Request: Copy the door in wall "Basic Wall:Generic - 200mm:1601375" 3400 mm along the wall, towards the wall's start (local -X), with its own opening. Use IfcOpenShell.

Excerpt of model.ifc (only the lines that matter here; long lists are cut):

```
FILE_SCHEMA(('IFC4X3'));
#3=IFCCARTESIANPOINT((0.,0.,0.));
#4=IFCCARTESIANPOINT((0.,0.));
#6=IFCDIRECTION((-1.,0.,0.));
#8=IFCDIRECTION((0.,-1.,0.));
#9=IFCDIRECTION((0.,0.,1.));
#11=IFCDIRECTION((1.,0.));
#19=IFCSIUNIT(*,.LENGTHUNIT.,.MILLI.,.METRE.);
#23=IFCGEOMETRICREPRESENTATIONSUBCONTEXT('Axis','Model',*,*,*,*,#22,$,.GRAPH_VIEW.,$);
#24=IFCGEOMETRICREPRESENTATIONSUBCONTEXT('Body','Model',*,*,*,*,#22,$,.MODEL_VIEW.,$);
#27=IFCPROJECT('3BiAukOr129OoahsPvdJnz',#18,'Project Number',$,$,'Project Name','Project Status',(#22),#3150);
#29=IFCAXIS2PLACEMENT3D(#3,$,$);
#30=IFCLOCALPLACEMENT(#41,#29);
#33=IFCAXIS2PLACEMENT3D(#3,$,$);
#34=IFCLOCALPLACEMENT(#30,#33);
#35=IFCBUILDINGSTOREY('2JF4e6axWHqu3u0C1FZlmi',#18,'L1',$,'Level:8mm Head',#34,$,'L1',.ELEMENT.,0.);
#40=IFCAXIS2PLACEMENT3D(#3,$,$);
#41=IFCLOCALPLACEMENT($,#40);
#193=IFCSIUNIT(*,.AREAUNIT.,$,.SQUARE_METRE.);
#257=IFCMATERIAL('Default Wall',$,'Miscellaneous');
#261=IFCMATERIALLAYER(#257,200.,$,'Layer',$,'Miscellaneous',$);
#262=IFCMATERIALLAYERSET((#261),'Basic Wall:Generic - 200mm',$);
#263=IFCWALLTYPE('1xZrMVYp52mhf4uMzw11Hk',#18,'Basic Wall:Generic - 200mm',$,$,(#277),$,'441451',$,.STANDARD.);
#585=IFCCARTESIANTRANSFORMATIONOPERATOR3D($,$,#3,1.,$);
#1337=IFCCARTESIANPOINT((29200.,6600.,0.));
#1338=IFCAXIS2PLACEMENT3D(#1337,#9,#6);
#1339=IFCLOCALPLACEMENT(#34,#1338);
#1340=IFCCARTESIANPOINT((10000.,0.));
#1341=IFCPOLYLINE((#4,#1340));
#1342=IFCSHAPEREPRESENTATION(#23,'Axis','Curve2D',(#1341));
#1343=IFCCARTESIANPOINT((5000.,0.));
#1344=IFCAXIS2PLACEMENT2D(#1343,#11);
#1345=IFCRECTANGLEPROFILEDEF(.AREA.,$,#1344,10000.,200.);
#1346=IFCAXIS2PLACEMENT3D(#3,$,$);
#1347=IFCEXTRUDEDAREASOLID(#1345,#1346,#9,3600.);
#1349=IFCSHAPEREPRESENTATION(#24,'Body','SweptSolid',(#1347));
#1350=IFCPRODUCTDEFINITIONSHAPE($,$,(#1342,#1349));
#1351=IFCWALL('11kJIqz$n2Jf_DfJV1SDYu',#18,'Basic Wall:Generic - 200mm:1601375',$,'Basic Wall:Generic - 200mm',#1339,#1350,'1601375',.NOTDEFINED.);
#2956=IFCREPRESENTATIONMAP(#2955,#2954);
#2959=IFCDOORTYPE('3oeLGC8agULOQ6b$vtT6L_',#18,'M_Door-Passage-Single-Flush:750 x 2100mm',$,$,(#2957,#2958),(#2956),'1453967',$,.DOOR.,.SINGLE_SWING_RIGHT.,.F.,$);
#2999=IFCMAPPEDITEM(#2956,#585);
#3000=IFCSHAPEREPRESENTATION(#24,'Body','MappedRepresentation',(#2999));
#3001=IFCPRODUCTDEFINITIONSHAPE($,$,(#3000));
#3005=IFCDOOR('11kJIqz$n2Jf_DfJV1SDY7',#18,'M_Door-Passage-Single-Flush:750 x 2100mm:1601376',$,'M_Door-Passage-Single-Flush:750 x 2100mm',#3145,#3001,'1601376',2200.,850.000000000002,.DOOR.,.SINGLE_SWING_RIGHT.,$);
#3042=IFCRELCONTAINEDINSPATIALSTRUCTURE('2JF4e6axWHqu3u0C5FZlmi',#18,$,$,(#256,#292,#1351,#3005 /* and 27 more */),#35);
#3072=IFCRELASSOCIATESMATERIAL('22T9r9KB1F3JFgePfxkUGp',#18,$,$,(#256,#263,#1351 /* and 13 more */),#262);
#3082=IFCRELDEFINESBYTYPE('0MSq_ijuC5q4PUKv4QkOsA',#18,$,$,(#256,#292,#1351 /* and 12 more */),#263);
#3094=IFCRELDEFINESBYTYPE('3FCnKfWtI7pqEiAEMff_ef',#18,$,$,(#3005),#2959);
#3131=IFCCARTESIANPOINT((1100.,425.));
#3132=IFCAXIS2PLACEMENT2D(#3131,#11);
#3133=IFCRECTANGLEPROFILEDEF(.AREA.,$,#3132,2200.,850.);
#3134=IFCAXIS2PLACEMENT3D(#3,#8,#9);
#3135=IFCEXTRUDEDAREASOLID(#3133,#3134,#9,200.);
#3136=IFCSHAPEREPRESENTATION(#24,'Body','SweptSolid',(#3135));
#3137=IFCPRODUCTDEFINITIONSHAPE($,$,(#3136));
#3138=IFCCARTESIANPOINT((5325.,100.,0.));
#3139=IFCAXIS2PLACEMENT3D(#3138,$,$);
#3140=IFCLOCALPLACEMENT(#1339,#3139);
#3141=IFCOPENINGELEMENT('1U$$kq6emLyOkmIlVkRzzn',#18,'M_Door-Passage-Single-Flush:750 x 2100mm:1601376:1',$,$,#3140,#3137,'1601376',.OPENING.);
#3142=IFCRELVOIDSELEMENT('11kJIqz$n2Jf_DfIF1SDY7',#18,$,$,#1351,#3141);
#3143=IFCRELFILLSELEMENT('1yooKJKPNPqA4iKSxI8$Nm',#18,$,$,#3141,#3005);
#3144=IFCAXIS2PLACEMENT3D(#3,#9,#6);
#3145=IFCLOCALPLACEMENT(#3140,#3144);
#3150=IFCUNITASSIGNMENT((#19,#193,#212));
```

```python
import ifcopenshell
import ifcopenshell.api.feature
import ifcopenshell.api.geometry
import ifcopenshell.api.root
import ifcopenshell.geom
import ifcopenshell.util.element
import ifcopenshell.util.placement
import ifcopenshell.util.shape

model = ifcopenshell.open("model.ifc")
settings = ifcopenshell.geom.settings()


def volume(element):
    """Net volume in cubic metres, openings subtracted."""
    shape = ifcopenshell.geom.create_shape(settings, element)
    return ifcopenshell.util.shape.get_volume(shape.geometry)


def reuse_history(source, copy):
    """copy_class also copies each property set's owner history, people and application; keep the originals."""
    for rel in copy.IsDefinedBy:
        if rel.is_a("IfcRelDefinesByProperties") and (history := rel.RelatingPropertyDefinition.OwnerHistory):
            rel.RelatingPropertyDefinition.OwnerHistory = source.OwnerHistory
            ifcopenshell.util.element.remove_deep2(model, history)


door = model.by_guid("11kJIqz$n2Jf_DfJV1SDY7")
opening = door.FillsVoids[0].RelatingOpeningElement
wall = opening.VoidsElements[0].RelatingBuildingElement
before = volume(wall)
shift = ifcopenshell.util.placement.get_local_placement(wall.ObjectPlacement)[:3, 0] * -3400.0

# copy_class copies the void relationship, type, container and properties, but no geometry.
new_opening = ifcopenshell.api.root.copy_class(model, product=opening)
new_opening.Representation = ifcopenshell.util.element.copy_deep(
    model, opening.Representation, exclude=["IfcGeometricRepresentationContext", "IfcRepresentationMap"]
)
new_opening.Name = "M_Door-Passage-Single-Flush:750 x 2100mm"
new_opening.Tag = None
new_door = ifcopenshell.api.root.copy_class(model, product=door)
new_door.Representation = ifcopenshell.util.element.copy_deep(
    model, door.Representation, exclude=["IfcGeometricRepresentationContext", "IfcRepresentationMap"]
)
new_door.Name = "M_Door-Passage-Single-Flush:750 x 2100mm"
new_door.Tag = None
reuse_history(door, new_door)
ifcopenshell.api.feature.add_filling(model, opening=new_opening, element=new_door)

for old, new in ((opening, new_opening), (door, new_door)):
    matrix = ifcopenshell.util.placement.get_local_placement(old.ObjectPlacement)
    matrix[:3, 3] += shift
    ifcopenshell.api.geometry.edit_object_placement(model, product=new, matrix=matrix, is_si=False)

after = volume(wall)

print(f"wall volume {before:.3f} -> {after:.3f} m3")

model.write("model_updated.ifc")
```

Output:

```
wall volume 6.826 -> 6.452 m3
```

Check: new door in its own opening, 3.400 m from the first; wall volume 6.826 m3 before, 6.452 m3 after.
